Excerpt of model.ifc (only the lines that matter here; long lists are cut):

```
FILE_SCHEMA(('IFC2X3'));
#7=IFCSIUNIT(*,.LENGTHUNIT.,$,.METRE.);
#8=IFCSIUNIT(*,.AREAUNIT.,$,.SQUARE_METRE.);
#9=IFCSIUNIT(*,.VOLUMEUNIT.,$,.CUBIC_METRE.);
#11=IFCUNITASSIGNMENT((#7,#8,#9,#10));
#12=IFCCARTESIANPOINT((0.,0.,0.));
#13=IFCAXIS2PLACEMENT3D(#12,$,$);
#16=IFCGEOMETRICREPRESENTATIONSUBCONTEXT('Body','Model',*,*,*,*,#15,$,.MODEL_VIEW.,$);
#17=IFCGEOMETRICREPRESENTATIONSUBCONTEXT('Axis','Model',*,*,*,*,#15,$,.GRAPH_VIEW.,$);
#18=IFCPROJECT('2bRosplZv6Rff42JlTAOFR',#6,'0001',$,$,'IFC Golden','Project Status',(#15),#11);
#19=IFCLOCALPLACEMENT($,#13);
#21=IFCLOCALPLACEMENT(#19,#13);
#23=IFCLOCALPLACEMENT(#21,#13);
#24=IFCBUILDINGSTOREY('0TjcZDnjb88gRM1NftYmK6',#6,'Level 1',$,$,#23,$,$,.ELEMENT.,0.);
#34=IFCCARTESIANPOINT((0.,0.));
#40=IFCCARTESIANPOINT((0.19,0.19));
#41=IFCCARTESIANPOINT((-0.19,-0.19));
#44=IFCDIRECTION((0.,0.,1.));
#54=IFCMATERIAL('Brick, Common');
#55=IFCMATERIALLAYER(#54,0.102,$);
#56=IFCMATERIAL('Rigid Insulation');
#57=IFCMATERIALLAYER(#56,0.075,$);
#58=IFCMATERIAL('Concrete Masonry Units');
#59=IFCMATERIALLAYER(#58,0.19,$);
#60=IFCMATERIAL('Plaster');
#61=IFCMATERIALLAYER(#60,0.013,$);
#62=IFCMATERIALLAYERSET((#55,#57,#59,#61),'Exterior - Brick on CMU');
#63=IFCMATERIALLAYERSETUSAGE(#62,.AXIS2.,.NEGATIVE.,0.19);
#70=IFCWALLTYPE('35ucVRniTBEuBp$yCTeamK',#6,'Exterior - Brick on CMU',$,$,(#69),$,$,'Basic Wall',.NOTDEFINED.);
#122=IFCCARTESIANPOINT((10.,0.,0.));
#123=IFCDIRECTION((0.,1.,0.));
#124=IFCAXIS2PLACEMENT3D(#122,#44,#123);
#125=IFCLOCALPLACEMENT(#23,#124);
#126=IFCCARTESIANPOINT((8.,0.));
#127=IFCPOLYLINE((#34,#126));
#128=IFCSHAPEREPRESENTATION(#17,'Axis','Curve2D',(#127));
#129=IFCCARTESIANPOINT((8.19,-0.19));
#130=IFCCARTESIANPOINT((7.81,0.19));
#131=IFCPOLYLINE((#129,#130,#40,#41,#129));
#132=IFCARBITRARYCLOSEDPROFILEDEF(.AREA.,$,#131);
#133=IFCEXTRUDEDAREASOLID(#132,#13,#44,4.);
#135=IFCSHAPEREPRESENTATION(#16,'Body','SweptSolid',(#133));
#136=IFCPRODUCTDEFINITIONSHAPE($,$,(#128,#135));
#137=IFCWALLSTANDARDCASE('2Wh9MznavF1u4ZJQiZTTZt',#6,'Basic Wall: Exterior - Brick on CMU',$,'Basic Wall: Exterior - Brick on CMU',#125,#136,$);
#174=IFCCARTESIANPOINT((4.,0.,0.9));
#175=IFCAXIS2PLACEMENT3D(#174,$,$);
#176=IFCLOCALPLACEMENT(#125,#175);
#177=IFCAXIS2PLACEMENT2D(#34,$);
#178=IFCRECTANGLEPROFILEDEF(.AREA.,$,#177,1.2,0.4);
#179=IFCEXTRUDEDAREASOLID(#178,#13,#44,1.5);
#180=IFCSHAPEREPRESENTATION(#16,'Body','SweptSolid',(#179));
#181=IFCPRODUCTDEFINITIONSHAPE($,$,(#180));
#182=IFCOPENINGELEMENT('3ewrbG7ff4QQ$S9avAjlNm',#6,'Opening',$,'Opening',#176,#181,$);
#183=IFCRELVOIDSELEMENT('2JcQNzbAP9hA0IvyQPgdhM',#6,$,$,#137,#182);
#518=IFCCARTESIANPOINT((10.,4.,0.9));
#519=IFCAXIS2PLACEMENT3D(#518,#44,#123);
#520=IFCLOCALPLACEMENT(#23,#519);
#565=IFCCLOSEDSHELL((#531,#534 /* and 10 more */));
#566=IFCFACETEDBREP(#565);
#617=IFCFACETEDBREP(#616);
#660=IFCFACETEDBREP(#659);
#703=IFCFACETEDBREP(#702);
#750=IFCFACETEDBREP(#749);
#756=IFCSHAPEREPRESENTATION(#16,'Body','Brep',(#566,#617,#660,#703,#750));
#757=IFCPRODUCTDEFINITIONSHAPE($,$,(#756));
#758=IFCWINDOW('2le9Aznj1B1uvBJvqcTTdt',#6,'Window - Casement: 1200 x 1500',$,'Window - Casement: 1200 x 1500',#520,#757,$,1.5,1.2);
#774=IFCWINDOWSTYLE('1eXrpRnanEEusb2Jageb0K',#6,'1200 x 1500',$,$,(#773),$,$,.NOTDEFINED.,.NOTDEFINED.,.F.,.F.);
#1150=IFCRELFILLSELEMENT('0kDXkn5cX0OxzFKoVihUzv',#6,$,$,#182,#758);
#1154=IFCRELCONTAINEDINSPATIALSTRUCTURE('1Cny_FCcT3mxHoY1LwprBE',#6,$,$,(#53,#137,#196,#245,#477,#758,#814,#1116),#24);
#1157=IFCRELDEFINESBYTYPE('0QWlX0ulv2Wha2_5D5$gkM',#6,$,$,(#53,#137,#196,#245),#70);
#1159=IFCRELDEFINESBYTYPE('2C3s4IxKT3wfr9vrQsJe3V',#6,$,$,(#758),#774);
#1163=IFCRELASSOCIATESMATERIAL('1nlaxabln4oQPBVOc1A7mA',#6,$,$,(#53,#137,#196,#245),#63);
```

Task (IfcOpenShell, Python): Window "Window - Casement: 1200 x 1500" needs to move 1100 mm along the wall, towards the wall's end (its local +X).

```python
import ifcopenshell
import ifcopenshell.api.geometry
import ifcopenshell.util.placement
import ifcopenshell.util.unit

model = ifcopenshell.open("model.ifc")
unit_scale = ifcopenshell.util.unit.calculate_unit_scale(model)

window = model.by_id(758)
opening = window.FillsVoids[0].RelatingOpeningElement
wall = opening.VoidsElements[0].RelatingBuildingElement

wall_matrix = ifcopenshell.util.placement.get_local_placement(wall.ObjectPlacement)
shift = wall_matrix[:3, 0] * 1.1 / unit_scale
before = ifcopenshell.util.placement.get_local_placement(window.ObjectPlacement)[:3, 3].copy()

# The window is not placed relative to its opening, so move both.
for product in (opening, window):
    matrix = ifcopenshell.util.placement.get_local_placement(product.ObjectPlacement)
    matrix[:3, 3] += shift
    ifcopenshell.api.geometry.edit_object_placement(model, product=product, matrix=matrix, is_si=False)

after = ifcopenshell.util.placement.get_local_placement(window.ObjectPlacement)[:3, 3]
print("window moved by", (after - before).round(3) + 0.0)

model.write("model_updated.ifc")
```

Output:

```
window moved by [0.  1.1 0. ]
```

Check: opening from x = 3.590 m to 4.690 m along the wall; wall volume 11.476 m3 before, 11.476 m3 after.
